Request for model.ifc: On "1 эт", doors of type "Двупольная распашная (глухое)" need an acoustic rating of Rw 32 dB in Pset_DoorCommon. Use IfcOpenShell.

First a look at what the model holds.

```python
import ifcopenshell
import ifcopenshell.util.element

model = ifcopenshell.open("model.ifc")
print(model.schema)
storey = next(s for s in model.by_type("IfcBuildingStorey") if s.Name == "1 эт")
doors = [e for e in ifcopenshell.util.element.get_decomposition(storey) if e.is_a("IfcDoor")]
seen = {}
for e in doors:
    element_type = ifcopenshell.util.element.get_type(e)
    key = (element_type.Name if element_type != e and element_type else None, ifcopenshell.util.element.get_pset(e, "Pset_DoorCommon", "AcousticRating"))
    seen[key] = seen.get(key, 0) + 1
for (name, value), count in sorted(seen.items(), key=str):
    print(count, "x", name, "|", value)
```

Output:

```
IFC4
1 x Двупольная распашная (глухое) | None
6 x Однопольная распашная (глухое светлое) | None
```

```python
import ifcopenshell
import ifcopenshell.api.pset
import ifcopenshell.util.element

model = ifcopenshell.open("model.ifc")

storey = next(s for s in model.by_type("IfcBuildingStorey") if s.Name == "1 эт")
doors = [e for e in ifcopenshell.util.element.get_decomposition(storey) if e.is_a("IfcDoor")]

count = 0
for e in doors:
    element_type = ifcopenshell.util.element.get_type(e)
    if element_type in (None, e) or element_type.Name != "Двупольная распашная (глухое)":
        continue
    # add_pset returns the element's existing set when there is one.
    pset = ifcopenshell.api.pset.add_pset(model, product=e, name="Pset_DoorCommon")
    ifcopenshell.api.pset.edit_pset(model, pset=pset, properties={"AcousticRating": "Rw 32 dB"})
    count += 1

print(count, "doors updated")

model.write("model-out.ifc")
```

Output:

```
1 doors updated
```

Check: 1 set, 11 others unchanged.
